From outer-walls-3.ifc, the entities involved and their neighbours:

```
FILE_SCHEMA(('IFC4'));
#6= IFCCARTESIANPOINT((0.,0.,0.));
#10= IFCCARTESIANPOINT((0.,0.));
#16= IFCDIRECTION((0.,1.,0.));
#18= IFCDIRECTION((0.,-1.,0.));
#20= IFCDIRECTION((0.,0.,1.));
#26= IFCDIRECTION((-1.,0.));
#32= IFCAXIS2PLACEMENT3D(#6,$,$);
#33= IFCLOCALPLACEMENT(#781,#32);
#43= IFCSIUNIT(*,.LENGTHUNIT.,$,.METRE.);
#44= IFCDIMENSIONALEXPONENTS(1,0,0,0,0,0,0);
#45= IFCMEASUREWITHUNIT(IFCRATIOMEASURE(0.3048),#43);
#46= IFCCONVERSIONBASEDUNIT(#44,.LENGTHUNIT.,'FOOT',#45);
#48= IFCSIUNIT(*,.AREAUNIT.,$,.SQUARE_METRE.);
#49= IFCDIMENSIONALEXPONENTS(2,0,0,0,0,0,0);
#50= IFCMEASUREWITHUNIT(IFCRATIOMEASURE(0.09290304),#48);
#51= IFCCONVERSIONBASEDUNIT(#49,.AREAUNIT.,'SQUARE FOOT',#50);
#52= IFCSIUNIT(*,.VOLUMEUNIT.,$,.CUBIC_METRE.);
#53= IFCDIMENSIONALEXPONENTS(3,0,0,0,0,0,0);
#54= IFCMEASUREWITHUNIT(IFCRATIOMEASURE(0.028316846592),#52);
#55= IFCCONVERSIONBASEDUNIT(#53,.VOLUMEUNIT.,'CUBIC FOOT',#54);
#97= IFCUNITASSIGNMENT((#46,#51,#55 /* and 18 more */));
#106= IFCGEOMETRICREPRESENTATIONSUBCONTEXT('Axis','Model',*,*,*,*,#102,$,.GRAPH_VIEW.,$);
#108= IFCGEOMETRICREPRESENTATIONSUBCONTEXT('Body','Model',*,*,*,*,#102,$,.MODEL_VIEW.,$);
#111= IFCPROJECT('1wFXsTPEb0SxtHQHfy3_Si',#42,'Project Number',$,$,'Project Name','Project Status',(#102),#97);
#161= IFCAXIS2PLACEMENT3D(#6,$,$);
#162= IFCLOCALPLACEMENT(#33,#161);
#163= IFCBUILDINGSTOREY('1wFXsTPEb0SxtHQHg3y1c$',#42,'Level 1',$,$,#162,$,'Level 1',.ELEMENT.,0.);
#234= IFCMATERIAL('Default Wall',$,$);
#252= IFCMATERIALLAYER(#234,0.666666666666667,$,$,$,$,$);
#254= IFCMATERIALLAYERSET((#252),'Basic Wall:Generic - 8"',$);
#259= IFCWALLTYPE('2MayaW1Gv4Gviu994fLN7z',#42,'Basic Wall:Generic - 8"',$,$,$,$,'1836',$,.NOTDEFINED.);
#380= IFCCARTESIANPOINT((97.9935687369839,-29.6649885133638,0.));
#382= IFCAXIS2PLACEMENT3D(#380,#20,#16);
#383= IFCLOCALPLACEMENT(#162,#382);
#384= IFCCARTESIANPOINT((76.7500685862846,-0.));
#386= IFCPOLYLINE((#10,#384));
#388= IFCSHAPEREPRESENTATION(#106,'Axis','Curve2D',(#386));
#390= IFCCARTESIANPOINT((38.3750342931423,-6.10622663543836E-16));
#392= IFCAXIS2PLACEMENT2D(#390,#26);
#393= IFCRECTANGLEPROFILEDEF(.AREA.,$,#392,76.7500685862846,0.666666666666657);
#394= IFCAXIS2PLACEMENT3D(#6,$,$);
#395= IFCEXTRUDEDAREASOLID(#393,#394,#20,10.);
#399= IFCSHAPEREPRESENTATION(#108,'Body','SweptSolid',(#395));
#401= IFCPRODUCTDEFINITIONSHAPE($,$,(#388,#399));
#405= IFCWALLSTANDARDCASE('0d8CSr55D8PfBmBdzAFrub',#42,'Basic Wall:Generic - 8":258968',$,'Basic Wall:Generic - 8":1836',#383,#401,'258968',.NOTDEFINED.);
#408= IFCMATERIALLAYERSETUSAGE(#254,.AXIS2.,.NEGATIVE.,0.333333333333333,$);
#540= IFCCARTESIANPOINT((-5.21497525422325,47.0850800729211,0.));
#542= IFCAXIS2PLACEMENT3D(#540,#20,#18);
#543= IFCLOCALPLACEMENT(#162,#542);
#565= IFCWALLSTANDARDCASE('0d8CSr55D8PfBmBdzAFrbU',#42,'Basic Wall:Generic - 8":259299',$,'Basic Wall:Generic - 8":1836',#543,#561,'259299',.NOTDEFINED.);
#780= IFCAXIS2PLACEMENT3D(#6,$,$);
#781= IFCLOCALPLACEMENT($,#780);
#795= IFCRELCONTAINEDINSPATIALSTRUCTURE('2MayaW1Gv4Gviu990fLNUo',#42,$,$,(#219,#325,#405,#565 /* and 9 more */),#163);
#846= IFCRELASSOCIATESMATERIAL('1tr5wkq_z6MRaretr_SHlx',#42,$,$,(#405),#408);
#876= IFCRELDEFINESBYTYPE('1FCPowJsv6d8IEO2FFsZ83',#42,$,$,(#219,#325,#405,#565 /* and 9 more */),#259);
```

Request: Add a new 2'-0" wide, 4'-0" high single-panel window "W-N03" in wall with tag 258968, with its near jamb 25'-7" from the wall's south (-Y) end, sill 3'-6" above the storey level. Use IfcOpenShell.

```python
import numpy as np
import ifcopenshell
import ifcopenshell.api.feature
import ifcopenshell.api.geometry
import ifcopenshell.api.root
import ifcopenshell.api.spatial
import ifcopenshell.geom
import ifcopenshell.util.element
import ifcopenshell.util.placement
import ifcopenshell.util.representation
import ifcopenshell.util.shape
import ifcopenshell.util.unit

model = ifcopenshell.open("outer-walls-3.ifc")
unit_scale = ifcopenshell.util.unit.calculate_unit_scale(model)
settings = ifcopenshell.geom.settings()


def volume(element):
    """Net volume in cubic metres, openings subtracted."""
    shape = ifcopenshell.geom.create_shape(settings, element)
    return ifcopenshell.util.shape.get_volume(shape.geometry)


wall = model.by_guid("0d8CSr55D8PfBmBdzAFrub")
storey = ifcopenshell.util.element.get_container(wall, ifc_class="IfcBuildingStorey")
context = ifcopenshell.util.representation.get_context(model, "Model", "Body", "MODEL_VIEW")
before = volume(wall)

width, height, from_end, sill = 0.6096, 1.2192, 7.7978, 1.0668  # metres

# The wall runs along its own X axis, and the end named is its -X end.
wall_shape = ifcopenshell.geom.create_shape(settings, wall)
x, y, z = ifcopenshell.util.shape.get_vertices(wall_shape.geometry).T
start = x.min() + from_end
face, thickness = float(y.min()), float(y.max() - y.min())
wall_matrix = ifcopenshell.util.placement.get_local_placement(wall.ObjectPlacement)
level = ifcopenshell.util.placement.get_local_placement(storey.ObjectPlacement)[2, 3]


def in_wall(x, y):
    """Placement at x, y metres in the wall's axes, at sill height."""
    matrix = wall_matrix.copy()
    matrix[:, 3] = wall_matrix @ np.array([x / unit_scale, y / unit_scale, 0.0, 1.0])
    matrix[2, 3] = level + sill / unit_scale
    return matrix


# Opening: a box that overshoots both wall faces by 50 mm.
opening = ifcopenshell.api.root.create_entity(model, ifc_class="IfcOpeningElement", predefined_type="OPENING")
box = ifcopenshell.api.geometry.add_wall_representation(
    model, context=context, length=width, height=height, thickness=thickness + 0.1
)
ifcopenshell.api.geometry.assign_representation(model, product=opening, representation=box)
ifcopenshell.api.geometry.edit_object_placement(model, product=opening, matrix=in_wall(start, face - 0.05), is_si=False)
ifcopenshell.api.feature.add_feature(model, feature=opening, element=wall)

window = ifcopenshell.api.root.create_entity(model, ifc_class="IfcWindow", name="W-N03", predefined_type="WINDOW")
window.OverallWidth, window.OverallHeight = width / unit_scale, height / unit_scale
window.PartitioningType = "SINGLE_PANEL"
body = ifcopenshell.api.geometry.add_window_representation(
    model,
    context=context,
    overall_width=window.OverallWidth,
    overall_height=window.OverallHeight,
    partition_type="SINGLE_PANEL",
)
ifcopenshell.api.geometry.assign_representation(model, product=window, representation=body)
ifcopenshell.api.spatial.assign_container(model, products=[window], relating_structure=storey)
ifcopenshell.api.feature.add_filling(model, opening=opening, element=window)

# Centre the window in the wall's thickness.
ifcopenshell.api.geometry.edit_object_placement(model, product=window, matrix=in_wall(start, face), is_si=False)
window_shape = ifcopenshell.geom.create_shape(settings, window)
depth = ifcopenshell.util.shape.get_vertices(window_shape.geometry)[:, 1]
offset = face + thickness / 2 - (depth.min() + depth.max()) / 2
ifcopenshell.api.geometry.edit_object_placement(model, product=window, matrix=in_wall(start, offset), is_si=False)

after = volume(wall)

print(f"wall volume {before:.3f} -> {after:.3f} m3")

model.write("outer-walls-3_updated.ifc")
```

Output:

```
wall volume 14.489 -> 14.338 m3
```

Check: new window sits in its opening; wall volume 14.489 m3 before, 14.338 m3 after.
